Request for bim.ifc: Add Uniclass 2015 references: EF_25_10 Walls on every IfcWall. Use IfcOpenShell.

First a look at what the model holds.

```python
import ifcopenshell

model = ifcopenshell.open("bim.ifc")
print(model.schema)
print("classifications:", [c.Name for c in model.by_type("IfcClassification")])
for ifc_class in ("IfcDoor", "IfcRoof", "IfcStair", "IfcWall", "IfcWindow"):
    print(ifc_class, len(model.by_type(ifc_class)))
```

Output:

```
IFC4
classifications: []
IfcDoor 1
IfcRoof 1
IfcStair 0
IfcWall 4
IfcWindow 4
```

```python
import ifcopenshell
import ifcopenshell.api.classification

model = ifcopenshell.open("bim.ifc")

system = ifcopenshell.api.classification.add_classification(model, classification="Uniclass 2015")

codes = {
    "IfcWall": ("EF_25_10", "Walls"),
}
for ifc_class, (code, name) in codes.items():
    products = model.by_type(ifc_class)
    ifcopenshell.api.classification.add_reference(
        model, products=products, classification=system, identification=code, name=name
    )
    print(code, len(products))

model.write("bim-out.ifc")
```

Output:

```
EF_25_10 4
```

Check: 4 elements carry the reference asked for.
